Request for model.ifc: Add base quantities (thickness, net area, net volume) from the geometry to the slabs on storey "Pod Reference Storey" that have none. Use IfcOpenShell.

First a look at what the model holds.

```python
import ifcopenshell
import ifcopenshell.util.element
import ifcopenshell.util.unit

model = ifcopenshell.open("model.ifc")
print(model.schema)
for unit_type in ("LENGTHUNIT", "AREAUNIT", "VOLUMEUNIT"):
    print(unit_type, ifcopenshell.util.unit.calculate_unit_scale(model, unit_type))
storey = next(s for s in model.by_type("IfcBuildingStorey") if s.Name == "Pod Reference Storey")
slabs = [e for e in ifcopenshell.util.element.get_decomposition(storey) if e.is_a("IfcSlab")]
for e in sorted(slabs, key=lambda e: e.id()):
    print(e.id(), e.is_a(), e.Name, list(ifcopenshell.util.element.get_psets(e, qtos_only=True)), sep=" | ")
```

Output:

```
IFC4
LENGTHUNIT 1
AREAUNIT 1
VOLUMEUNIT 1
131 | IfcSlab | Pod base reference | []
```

```python
import ifcopenshell
import ifcopenshell.api.pset
import ifcopenshell.geom
import ifcopenshell.util.element
import ifcopenshell.util.shape
import ifcopenshell.util.unit

model = ifcopenshell.open("model.ifc")
unit_scale = ifcopenshell.util.unit.calculate_unit_scale(model)
area_scale = ifcopenshell.util.unit.calculate_unit_scale(model, "AREAUNIT")
volume_scale = ifcopenshell.util.unit.calculate_unit_scale(model, "VOLUMEUNIT")
settings = ifcopenshell.geom.settings()

storey = next(s for s in model.by_type("IfcBuildingStorey") if s.Name == "Pod Reference Storey")
slabs = [e for e in ifcopenshell.util.element.get_decomposition(storey) if e.is_a("IfcSlab")]

for e in sorted(slabs, key=lambda e: e.id()):
    if ifcopenshell.util.element.get_psets(e, qtos_only=True, should_inherit=False):
        continue
    # Geometry comes back in metres, in the element's own axes.
    shape = ifcopenshell.geom.create_shape(settings, e)
    values = {
        "Width": ifcopenshell.util.shape.get_z(shape.geometry) / unit_scale,
        "NetArea": ifcopenshell.util.shape.get_footprint_area(shape.geometry) / area_scale,
        "NetVolume": ifcopenshell.util.shape.get_volume(shape.geometry) / volume_scale,
    }
    qto = ifcopenshell.api.pset.add_qto(model, product=e, name="Qto_SlabBaseQuantities")
    ifcopenshell.api.pset.edit_qto(model, qto=qto, properties=values)
    print(e.id(), {k: round(v, 3) for k, v in values.items()})

model.write("model-out.ifc")
```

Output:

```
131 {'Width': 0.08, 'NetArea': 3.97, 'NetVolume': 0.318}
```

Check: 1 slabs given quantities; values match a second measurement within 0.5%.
